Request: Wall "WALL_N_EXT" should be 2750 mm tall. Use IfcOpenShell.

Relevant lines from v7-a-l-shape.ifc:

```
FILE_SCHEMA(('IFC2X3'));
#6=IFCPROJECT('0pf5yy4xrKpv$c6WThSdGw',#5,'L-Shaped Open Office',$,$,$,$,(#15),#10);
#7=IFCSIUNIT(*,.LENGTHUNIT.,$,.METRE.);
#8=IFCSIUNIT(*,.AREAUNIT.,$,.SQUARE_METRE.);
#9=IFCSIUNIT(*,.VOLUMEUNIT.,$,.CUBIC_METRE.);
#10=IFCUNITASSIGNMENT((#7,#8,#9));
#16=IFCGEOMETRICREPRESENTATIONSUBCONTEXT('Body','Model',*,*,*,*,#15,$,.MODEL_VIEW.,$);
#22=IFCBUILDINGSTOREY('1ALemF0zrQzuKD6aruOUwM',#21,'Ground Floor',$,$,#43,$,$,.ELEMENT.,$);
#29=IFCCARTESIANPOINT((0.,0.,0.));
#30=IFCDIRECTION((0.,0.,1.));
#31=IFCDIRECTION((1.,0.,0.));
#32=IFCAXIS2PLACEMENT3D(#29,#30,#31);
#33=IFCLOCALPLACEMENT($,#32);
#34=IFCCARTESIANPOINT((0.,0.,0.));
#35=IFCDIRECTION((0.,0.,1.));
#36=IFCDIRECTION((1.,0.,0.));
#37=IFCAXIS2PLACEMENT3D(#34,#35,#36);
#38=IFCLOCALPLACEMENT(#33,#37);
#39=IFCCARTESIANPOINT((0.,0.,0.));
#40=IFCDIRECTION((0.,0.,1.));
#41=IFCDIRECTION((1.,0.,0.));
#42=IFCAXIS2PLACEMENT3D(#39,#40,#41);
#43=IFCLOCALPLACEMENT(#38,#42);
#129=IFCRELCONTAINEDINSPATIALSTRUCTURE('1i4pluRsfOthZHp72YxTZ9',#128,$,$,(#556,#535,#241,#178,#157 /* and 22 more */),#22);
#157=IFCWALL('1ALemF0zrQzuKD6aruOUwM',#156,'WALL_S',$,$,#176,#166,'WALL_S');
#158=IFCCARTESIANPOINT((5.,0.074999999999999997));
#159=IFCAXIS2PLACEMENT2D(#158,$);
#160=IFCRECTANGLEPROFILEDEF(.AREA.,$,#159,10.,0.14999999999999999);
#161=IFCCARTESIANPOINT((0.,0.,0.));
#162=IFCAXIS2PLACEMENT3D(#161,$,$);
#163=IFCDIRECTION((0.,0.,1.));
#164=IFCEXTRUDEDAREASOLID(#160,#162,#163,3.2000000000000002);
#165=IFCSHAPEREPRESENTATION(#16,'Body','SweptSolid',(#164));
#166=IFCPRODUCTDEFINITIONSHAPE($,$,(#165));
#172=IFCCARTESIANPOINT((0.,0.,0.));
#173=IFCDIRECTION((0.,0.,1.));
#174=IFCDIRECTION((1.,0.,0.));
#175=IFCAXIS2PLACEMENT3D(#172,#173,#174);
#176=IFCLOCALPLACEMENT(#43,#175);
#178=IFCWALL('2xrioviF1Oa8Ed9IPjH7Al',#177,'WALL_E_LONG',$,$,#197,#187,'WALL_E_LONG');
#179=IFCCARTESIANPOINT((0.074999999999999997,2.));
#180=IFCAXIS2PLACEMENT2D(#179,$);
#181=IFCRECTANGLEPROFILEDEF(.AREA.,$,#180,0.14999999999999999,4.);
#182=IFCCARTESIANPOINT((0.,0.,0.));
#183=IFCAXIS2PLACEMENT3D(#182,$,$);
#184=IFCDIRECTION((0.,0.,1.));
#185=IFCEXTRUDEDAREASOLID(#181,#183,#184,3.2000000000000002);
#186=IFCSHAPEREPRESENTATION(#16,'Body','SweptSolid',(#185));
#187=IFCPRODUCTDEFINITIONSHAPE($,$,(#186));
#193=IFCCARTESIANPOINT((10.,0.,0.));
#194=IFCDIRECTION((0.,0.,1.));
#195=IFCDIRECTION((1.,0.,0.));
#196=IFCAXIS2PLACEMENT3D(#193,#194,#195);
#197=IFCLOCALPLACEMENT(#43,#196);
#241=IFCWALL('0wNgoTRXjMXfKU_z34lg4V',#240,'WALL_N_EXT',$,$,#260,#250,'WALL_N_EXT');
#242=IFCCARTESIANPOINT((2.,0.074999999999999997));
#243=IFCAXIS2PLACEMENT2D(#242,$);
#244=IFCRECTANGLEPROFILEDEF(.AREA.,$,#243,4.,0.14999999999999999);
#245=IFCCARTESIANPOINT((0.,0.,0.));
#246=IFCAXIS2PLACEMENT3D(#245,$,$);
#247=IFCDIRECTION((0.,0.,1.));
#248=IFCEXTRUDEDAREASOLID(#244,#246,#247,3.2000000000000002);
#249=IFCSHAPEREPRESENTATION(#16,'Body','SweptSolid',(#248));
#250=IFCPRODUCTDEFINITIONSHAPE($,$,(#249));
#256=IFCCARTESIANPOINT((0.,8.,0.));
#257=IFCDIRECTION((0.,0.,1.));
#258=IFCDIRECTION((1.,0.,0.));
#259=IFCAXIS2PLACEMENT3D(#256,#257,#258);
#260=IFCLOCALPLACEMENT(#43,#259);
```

```python
import ifcopenshell
import ifcopenshell.geom
import ifcopenshell.util.representation
import ifcopenshell.util.shape
import ifcopenshell.util.unit

model = ifcopenshell.open("v7-a-l-shape.ifc")
unit_scale = ifcopenshell.util.unit.calculate_unit_scale(model)
settings = ifcopenshell.geom.settings()


def volume(element):
    """Net volume in cubic metres, openings subtracted."""
    shape = ifcopenshell.geom.create_shape(settings, element)
    return ifcopenshell.util.shape.get_volume(shape.geometry)


wall = model.by_id(241)
before = volume(wall)

body = ifcopenshell.util.representation.get_representation(wall, "Model", "Body")
solid = body.Items[0]
old_height = solid.Depth
solid.Depth = 2.75 / unit_scale
after = volume(wall)

print(f"height {old_height:g} -> {solid.Depth:g}, volume {before:.3f} -> {after:.3f} m3")

model.write("v7-a-l-shape_v2.ifc")
```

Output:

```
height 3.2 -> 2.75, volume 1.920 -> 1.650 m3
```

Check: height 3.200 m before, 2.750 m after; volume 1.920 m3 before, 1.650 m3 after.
